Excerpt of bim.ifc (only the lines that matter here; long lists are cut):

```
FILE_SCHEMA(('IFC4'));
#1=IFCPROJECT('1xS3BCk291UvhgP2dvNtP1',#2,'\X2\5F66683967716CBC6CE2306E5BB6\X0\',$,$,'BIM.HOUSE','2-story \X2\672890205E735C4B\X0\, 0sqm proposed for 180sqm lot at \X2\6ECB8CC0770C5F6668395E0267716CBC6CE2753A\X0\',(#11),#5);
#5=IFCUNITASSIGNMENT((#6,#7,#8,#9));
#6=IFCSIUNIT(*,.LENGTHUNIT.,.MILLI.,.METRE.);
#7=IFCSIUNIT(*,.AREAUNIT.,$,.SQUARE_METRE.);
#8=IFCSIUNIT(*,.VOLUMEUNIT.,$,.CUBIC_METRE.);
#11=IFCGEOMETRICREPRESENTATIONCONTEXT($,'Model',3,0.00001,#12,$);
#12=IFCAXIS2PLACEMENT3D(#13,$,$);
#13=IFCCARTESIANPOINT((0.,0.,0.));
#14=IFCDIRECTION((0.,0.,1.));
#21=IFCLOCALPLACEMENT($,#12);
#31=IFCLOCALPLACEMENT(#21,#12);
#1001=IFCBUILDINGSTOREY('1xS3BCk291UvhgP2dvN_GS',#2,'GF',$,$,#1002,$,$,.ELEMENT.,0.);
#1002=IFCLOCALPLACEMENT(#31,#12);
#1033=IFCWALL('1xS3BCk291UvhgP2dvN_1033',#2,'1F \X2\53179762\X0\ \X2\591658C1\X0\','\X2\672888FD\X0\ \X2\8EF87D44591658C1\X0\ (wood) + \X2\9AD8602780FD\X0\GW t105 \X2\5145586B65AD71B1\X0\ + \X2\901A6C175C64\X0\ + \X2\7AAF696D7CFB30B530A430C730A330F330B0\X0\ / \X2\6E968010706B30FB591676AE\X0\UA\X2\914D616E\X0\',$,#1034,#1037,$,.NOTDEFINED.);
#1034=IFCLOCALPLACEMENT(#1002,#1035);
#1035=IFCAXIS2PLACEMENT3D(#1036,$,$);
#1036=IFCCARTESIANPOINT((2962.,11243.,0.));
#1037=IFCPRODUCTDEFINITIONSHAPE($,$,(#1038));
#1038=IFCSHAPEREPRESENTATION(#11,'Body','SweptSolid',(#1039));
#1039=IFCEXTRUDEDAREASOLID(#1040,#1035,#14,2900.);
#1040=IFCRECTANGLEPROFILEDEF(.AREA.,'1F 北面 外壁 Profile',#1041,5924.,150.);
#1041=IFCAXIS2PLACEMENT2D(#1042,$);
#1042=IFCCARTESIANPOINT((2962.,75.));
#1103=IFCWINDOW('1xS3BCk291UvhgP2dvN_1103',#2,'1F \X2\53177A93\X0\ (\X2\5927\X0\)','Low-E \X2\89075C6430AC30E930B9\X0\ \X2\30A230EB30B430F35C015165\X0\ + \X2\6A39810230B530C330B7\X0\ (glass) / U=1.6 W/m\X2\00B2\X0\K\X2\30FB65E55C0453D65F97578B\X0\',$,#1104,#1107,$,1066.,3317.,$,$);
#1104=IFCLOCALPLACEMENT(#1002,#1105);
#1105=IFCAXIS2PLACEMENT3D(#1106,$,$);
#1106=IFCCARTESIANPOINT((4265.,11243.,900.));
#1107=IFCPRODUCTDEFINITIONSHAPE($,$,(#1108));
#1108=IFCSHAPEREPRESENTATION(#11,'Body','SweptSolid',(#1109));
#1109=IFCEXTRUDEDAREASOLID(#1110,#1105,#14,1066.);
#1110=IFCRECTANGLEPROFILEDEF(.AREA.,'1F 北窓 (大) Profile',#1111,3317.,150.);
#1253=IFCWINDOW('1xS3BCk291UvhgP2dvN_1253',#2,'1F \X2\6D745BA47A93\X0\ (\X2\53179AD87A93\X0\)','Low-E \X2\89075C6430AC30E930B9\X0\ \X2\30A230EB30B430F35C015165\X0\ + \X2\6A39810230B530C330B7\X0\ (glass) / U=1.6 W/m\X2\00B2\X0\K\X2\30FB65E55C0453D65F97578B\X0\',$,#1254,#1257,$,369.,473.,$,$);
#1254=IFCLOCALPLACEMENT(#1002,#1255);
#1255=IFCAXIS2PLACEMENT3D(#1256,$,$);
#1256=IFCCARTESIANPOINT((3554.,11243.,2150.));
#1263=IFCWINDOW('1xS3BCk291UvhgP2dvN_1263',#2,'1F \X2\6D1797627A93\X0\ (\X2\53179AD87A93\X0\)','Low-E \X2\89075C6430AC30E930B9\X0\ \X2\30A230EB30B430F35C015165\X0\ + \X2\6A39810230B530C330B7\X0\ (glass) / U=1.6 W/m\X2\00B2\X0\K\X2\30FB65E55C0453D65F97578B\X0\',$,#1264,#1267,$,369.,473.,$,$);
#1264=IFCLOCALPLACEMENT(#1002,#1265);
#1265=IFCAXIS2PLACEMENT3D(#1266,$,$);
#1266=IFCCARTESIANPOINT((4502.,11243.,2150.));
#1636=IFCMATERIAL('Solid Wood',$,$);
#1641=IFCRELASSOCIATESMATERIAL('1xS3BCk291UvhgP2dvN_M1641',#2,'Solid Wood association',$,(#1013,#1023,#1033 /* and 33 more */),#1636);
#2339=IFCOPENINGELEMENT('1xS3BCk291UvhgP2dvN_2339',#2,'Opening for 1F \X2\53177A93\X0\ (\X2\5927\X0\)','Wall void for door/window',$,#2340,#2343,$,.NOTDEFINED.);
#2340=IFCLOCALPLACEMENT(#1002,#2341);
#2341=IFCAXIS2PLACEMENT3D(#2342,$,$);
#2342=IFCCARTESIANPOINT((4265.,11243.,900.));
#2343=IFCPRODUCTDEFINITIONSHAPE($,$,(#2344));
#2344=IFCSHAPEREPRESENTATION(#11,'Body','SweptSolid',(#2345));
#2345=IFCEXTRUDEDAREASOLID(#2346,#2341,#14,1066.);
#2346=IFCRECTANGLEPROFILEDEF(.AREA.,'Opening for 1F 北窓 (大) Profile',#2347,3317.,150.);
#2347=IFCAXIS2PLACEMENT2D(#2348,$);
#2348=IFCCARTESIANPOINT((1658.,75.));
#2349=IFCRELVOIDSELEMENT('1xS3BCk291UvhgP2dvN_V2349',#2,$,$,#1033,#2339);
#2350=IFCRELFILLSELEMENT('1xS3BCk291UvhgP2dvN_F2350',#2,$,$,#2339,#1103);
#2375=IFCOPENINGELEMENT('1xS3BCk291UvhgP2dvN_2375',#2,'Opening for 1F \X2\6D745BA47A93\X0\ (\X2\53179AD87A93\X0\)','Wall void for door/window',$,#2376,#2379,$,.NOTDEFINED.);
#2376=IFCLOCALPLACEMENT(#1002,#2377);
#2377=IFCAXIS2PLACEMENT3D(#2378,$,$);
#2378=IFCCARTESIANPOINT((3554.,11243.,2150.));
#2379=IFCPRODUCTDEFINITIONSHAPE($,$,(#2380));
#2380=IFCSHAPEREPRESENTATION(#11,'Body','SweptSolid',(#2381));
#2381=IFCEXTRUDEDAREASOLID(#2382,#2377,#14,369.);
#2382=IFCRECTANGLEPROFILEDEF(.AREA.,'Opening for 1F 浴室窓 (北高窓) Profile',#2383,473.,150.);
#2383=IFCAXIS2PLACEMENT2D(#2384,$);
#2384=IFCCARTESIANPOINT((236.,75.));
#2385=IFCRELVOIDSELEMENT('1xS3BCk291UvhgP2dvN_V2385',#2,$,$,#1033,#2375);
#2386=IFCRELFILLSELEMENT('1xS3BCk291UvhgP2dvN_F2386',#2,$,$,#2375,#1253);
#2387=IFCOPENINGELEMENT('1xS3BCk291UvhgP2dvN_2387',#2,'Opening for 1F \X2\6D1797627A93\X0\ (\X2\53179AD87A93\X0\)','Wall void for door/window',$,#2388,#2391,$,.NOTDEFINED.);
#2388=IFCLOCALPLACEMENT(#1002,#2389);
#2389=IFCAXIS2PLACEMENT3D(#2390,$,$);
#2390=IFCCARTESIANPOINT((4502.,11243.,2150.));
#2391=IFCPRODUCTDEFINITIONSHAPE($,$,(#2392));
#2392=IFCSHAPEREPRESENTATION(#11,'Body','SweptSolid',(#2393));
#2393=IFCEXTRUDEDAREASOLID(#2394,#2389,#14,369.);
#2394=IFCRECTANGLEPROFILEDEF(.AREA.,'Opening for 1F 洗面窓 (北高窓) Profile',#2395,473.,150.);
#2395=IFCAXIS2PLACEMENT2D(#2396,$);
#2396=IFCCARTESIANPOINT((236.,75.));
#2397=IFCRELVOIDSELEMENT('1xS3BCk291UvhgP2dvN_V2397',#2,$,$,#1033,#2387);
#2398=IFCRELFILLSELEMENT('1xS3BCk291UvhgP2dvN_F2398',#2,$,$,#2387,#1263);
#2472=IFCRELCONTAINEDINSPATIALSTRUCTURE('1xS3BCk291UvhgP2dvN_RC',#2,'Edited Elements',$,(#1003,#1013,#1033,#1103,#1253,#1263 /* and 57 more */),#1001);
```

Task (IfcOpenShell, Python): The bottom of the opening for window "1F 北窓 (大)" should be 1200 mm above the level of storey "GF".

```python
import numpy as np
import ifcopenshell
import ifcopenshell.api.geometry
import ifcopenshell.geom
import ifcopenshell.util.element
import ifcopenshell.util.placement
import ifcopenshell.util.shape
import ifcopenshell.util.unit

model = ifcopenshell.open("bim.ifc")
unit_scale = ifcopenshell.util.unit.calculate_unit_scale(model)

window = model.by_guid("1xS3BCk291UvhgP2dvN_1103")
opening = window.FillsVoids[0].RelatingOpeningElement
storey = ifcopenshell.util.element.get_container(window, ifc_class="IfcBuildingStorey")
level = ifcopenshell.util.placement.get_local_placement(storey.ObjectPlacement)[2, 3]

# The opening's origin need not be at the sill, so measure its lowest point.
shape = ifcopenshell.geom.create_shape(ifcopenshell.geom.settings(), opening)
bottom = ifcopenshell.util.shape.get_shape_bottom_elevation(shape, shape.geometry) / unit_scale
dz = level + 1.2 / unit_scale - bottom

shift = np.array([0.0, 0.0, dz])
# The window is not placed relative to its opening, so move both.
for product in (opening, window):
    matrix = ifcopenshell.util.placement.get_local_placement(product.ObjectPlacement)
    matrix[:3, 3] += shift
    ifcopenshell.api.geometry.edit_object_placement(model, product=product, matrix=matrix, is_si=False)

print(f"moved by {dz * unit_scale:+.3f} m")

model.write("bim_edited.ifc")
```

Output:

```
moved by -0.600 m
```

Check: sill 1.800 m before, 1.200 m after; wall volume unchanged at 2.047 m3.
